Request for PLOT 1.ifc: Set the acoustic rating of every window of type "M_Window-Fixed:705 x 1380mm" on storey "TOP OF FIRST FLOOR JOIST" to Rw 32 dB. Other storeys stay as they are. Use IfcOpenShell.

First a look at what the model holds.

```python
import ifcopenshell
import ifcopenshell.util.element

model = ifcopenshell.open("PLOT 1.ifc")
print(model.schema)
storey = next(s for s in model.by_type("IfcBuildingStorey") if s.Name == "TOP OF FIRST FLOOR JOIST")
windows = [e for e in ifcopenshell.util.element.get_decomposition(storey) if e.is_a("IfcWindow")]
seen = {}
for e in windows:
    element_type = ifcopenshell.util.element.get_type(e)
    key = (element_type.Name if element_type != e and element_type else None, ifcopenshell.util.element.get_pset(e, "Pset_WindowCommon", "AcousticRating"))
    seen[key] = seen.get(key, 0) + 1
for (name, value), count in sorted(seen.items(), key=str):
    print(count, "x", name, "|", value)
```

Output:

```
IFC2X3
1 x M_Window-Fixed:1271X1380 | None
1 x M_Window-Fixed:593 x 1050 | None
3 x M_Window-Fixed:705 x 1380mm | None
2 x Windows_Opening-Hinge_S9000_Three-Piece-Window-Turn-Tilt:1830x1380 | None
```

```python
import ifcopenshell
import ifcopenshell.api.pset
import ifcopenshell.util.element

model = ifcopenshell.open("PLOT 1.ifc")

storey = next(s for s in model.by_type("IfcBuildingStorey") if s.Name == "TOP OF FIRST FLOOR JOIST")
windows = [e for e in ifcopenshell.util.element.get_decomposition(storey) if e.is_a("IfcWindow")]

count = 0
for e in windows:
    element_type = ifcopenshell.util.element.get_type(e)
    if element_type in (None, e) or element_type.Name != "M_Window-Fixed:705 x 1380mm":
        continue
    # add_pset returns the element's existing set when there is one.
    pset = ifcopenshell.api.pset.add_pset(model, product=e, name="Pset_WindowCommon")
    ifcopenshell.api.pset.edit_pset(model, pset=pset, properties={"AcousticRating": "Rw 32 dB"})
    count += 1

print(count, "windows updated")

model.write("PLOT 1_updated.ifc")
```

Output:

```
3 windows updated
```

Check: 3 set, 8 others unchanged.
